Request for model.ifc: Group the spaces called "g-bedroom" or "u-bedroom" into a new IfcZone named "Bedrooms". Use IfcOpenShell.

First a look at what the model holds.

```python
import ifcopenshell

model = ifcopenshell.open("model.ifc")
print(model.schema)
seen = {}
for space in model.by_type("IfcSpace"):
    seen[space.LongName] = seen.get(space.LongName, 0) + 1
for name, count in sorted(seen.items(), key=str):
    print(count, "x", name)
print("zones:", [z.Name for z in model.by_type("IfcZone")][:20])
```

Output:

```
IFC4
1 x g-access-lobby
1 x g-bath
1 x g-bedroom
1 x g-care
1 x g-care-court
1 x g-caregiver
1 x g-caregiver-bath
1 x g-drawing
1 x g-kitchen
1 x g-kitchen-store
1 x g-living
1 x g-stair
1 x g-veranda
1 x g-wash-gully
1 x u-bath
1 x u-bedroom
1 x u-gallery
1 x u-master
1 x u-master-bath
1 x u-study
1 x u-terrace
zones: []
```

```python
import ifcopenshell
import ifcopenshell.api.group
import ifcopenshell.api.root

model = ifcopenshell.open("model.ifc")

names = {"g-bedroom", "u-bedroom"}
spaces = [s for s in model.by_type("IfcSpace") if s.LongName in names]

zone = ifcopenshell.api.root.create_entity(model, ifc_class="IfcZone", name="Bedrooms")
ifcopenshell.api.group.assign_group(model, products=spaces, group=zone)
print(len(spaces), "spaces in", zone.Name)

model.write("model-out.ifc")
```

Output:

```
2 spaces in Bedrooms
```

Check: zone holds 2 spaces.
